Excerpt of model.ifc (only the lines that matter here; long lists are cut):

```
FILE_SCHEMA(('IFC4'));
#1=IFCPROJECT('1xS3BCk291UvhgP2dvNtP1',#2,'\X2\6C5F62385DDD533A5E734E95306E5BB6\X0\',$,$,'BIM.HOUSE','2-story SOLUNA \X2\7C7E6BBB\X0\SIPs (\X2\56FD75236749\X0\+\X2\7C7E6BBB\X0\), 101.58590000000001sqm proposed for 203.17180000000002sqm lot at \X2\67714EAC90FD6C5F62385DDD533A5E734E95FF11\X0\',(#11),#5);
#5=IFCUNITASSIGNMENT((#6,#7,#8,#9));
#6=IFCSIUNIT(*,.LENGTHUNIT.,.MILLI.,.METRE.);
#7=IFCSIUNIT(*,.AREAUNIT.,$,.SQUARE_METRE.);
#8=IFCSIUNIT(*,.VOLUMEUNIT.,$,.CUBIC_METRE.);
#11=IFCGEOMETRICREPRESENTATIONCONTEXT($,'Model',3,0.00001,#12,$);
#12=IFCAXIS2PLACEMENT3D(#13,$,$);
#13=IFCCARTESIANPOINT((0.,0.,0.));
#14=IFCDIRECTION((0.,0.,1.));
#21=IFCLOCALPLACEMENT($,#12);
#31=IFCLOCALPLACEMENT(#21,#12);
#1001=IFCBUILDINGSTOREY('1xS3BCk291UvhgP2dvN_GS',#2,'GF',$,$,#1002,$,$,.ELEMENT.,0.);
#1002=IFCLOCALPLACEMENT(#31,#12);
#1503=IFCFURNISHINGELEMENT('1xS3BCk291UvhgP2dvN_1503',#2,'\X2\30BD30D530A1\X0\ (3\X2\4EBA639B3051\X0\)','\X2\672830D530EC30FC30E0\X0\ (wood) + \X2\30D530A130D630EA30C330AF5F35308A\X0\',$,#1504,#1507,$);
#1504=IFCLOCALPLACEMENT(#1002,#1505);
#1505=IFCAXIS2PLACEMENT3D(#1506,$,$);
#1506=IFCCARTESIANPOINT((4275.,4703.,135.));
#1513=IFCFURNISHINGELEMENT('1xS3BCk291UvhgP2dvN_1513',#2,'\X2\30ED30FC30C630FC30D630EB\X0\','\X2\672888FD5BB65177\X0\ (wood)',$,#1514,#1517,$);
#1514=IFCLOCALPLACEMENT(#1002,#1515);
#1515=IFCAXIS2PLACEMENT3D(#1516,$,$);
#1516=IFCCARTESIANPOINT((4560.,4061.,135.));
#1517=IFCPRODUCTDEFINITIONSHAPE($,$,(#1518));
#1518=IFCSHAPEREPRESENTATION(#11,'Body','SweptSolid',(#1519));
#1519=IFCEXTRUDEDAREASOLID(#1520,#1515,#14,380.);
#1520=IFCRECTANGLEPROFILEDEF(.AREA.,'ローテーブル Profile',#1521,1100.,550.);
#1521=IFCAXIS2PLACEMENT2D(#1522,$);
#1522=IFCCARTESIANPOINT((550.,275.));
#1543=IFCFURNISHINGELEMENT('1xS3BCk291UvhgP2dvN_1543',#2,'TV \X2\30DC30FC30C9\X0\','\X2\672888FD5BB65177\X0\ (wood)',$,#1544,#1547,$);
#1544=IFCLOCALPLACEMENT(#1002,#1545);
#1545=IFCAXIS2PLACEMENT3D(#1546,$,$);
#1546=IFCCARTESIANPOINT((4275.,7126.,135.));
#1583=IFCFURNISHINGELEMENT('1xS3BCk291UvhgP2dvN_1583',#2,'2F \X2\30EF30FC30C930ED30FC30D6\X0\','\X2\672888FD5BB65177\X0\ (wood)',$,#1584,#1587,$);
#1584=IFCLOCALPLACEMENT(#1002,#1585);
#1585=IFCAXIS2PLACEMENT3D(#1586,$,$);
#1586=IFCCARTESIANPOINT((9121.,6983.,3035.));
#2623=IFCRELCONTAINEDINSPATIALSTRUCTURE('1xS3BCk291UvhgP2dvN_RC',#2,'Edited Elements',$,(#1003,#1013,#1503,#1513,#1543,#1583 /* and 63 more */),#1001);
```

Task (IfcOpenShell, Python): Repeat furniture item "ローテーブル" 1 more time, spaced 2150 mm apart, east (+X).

```python
import numpy as np
import ifcopenshell
import ifcopenshell.api.geometry
import ifcopenshell.api.root
import ifcopenshell.util.element
import ifcopenshell.util.placement

model = ifcopenshell.open("model.ifc")


def reuse_history(source, copy):
    """copy_class also copies each property set's owner history, people and application; keep the originals."""
    for rel in copy.IsDefinedBy:
        if rel.is_a("IfcRelDefinesByProperties") and (history := rel.RelatingPropertyDefinition.OwnerHistory):
            rel.RelatingPropertyDefinition.OwnerHistory = source.OwnerHistory
            ifcopenshell.util.element.remove_deep2(model, history)


source = model.by_id(1513)
base = ifcopenshell.util.placement.get_local_placement(source.ObjectPlacement)
step = np.array([1.0, 0.0, 0.0]) * 2150.0

for i in range(1, 2):
    copy = ifcopenshell.api.root.copy_class(model, product=source)
    copy.Representation = ifcopenshell.util.element.copy_deep(
        model, source.Representation, exclude=["IfcGeometricRepresentationContext", "IfcRepresentationMap"]
    )
    reuse_history(source, copy)
    matrix = base.copy()
    matrix[:3, 3] += i * step
    print("added at", matrix[:3, 3].round(3) + 0.0)
    ifcopenshell.api.geometry.edit_object_placement(model, product=copy, matrix=matrix, is_si=False)

model.write("model_rev.ifc")
```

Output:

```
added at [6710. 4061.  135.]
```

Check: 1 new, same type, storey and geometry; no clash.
